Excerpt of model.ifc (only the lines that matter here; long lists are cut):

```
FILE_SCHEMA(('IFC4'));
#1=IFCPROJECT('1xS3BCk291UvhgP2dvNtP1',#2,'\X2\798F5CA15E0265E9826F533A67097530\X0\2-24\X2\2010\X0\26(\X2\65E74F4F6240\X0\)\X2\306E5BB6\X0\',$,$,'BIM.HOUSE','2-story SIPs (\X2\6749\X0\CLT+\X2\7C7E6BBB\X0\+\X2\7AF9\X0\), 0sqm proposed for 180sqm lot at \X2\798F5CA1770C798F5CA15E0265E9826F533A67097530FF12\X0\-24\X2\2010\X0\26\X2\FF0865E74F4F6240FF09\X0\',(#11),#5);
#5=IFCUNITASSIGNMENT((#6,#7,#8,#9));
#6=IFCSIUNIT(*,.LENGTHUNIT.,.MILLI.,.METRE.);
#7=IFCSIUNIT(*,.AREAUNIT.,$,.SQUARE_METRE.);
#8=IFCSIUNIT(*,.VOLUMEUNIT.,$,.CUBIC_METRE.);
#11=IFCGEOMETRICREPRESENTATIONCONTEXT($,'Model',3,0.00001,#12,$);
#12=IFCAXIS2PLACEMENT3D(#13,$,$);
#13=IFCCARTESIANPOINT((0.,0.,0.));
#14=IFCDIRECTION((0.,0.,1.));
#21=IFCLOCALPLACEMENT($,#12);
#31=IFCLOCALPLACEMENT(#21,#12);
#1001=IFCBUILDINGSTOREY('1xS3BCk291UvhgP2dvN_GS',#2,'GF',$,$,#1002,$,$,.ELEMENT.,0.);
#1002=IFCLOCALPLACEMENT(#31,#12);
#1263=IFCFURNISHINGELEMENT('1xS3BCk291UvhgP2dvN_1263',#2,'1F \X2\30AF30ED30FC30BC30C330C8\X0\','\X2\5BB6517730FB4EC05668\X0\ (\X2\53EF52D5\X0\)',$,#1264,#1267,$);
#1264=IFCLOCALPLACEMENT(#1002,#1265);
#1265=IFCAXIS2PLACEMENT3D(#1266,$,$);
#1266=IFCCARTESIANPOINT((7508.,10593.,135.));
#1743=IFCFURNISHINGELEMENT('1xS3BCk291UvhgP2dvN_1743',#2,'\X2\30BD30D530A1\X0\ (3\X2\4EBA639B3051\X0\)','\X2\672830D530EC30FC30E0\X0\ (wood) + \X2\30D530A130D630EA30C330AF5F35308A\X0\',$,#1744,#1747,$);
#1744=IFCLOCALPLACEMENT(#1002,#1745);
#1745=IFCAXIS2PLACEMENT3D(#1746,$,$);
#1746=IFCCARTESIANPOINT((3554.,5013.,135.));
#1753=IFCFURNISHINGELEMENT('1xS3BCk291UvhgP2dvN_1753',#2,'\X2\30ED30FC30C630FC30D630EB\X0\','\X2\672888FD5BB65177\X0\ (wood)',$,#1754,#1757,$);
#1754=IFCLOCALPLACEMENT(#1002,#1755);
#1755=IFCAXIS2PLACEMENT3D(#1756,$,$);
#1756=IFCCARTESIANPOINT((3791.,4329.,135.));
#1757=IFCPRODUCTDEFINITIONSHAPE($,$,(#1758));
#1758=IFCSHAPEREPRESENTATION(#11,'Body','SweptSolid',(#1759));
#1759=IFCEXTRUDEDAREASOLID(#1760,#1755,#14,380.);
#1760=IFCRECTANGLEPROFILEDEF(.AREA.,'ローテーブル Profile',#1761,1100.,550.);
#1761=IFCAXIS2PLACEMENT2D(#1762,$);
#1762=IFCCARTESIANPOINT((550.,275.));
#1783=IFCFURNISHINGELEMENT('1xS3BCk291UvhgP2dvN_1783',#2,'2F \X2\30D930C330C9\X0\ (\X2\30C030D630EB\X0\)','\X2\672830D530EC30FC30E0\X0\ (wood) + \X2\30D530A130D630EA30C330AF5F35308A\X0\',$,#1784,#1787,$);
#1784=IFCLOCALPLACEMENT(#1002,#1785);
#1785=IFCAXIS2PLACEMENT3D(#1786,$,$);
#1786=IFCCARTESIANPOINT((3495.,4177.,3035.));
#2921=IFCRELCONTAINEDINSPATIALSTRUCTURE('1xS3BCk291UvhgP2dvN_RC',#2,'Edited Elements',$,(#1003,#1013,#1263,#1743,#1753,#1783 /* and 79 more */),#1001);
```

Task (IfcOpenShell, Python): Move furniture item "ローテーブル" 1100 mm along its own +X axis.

```python
import ifcopenshell
import ifcopenshell.api.geometry
import ifcopenshell.util.placement
import ifcopenshell.util.unit

model = ifcopenshell.open("model.ifc")
unit_scale = ifcopenshell.util.unit.calculate_unit_scale(model)

item = model.by_id(1753)
matrix = ifcopenshell.util.placement.get_local_placement(item.ObjectPlacement)
matrix[:3, 3] += matrix[:3, 0] * 1.1 / unit_scale
ifcopenshell.api.geometry.edit_object_placement(model, product=item, matrix=matrix, is_si=False)

print(ifcopenshell.util.placement.get_local_placement(item.ObjectPlacement).round(3) + 0.0)

model.write("model_updated.ifc")
```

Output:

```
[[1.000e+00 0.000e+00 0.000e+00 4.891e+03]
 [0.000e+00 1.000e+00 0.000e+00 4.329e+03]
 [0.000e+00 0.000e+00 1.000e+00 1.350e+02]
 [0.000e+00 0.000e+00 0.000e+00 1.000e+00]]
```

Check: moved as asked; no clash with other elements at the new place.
